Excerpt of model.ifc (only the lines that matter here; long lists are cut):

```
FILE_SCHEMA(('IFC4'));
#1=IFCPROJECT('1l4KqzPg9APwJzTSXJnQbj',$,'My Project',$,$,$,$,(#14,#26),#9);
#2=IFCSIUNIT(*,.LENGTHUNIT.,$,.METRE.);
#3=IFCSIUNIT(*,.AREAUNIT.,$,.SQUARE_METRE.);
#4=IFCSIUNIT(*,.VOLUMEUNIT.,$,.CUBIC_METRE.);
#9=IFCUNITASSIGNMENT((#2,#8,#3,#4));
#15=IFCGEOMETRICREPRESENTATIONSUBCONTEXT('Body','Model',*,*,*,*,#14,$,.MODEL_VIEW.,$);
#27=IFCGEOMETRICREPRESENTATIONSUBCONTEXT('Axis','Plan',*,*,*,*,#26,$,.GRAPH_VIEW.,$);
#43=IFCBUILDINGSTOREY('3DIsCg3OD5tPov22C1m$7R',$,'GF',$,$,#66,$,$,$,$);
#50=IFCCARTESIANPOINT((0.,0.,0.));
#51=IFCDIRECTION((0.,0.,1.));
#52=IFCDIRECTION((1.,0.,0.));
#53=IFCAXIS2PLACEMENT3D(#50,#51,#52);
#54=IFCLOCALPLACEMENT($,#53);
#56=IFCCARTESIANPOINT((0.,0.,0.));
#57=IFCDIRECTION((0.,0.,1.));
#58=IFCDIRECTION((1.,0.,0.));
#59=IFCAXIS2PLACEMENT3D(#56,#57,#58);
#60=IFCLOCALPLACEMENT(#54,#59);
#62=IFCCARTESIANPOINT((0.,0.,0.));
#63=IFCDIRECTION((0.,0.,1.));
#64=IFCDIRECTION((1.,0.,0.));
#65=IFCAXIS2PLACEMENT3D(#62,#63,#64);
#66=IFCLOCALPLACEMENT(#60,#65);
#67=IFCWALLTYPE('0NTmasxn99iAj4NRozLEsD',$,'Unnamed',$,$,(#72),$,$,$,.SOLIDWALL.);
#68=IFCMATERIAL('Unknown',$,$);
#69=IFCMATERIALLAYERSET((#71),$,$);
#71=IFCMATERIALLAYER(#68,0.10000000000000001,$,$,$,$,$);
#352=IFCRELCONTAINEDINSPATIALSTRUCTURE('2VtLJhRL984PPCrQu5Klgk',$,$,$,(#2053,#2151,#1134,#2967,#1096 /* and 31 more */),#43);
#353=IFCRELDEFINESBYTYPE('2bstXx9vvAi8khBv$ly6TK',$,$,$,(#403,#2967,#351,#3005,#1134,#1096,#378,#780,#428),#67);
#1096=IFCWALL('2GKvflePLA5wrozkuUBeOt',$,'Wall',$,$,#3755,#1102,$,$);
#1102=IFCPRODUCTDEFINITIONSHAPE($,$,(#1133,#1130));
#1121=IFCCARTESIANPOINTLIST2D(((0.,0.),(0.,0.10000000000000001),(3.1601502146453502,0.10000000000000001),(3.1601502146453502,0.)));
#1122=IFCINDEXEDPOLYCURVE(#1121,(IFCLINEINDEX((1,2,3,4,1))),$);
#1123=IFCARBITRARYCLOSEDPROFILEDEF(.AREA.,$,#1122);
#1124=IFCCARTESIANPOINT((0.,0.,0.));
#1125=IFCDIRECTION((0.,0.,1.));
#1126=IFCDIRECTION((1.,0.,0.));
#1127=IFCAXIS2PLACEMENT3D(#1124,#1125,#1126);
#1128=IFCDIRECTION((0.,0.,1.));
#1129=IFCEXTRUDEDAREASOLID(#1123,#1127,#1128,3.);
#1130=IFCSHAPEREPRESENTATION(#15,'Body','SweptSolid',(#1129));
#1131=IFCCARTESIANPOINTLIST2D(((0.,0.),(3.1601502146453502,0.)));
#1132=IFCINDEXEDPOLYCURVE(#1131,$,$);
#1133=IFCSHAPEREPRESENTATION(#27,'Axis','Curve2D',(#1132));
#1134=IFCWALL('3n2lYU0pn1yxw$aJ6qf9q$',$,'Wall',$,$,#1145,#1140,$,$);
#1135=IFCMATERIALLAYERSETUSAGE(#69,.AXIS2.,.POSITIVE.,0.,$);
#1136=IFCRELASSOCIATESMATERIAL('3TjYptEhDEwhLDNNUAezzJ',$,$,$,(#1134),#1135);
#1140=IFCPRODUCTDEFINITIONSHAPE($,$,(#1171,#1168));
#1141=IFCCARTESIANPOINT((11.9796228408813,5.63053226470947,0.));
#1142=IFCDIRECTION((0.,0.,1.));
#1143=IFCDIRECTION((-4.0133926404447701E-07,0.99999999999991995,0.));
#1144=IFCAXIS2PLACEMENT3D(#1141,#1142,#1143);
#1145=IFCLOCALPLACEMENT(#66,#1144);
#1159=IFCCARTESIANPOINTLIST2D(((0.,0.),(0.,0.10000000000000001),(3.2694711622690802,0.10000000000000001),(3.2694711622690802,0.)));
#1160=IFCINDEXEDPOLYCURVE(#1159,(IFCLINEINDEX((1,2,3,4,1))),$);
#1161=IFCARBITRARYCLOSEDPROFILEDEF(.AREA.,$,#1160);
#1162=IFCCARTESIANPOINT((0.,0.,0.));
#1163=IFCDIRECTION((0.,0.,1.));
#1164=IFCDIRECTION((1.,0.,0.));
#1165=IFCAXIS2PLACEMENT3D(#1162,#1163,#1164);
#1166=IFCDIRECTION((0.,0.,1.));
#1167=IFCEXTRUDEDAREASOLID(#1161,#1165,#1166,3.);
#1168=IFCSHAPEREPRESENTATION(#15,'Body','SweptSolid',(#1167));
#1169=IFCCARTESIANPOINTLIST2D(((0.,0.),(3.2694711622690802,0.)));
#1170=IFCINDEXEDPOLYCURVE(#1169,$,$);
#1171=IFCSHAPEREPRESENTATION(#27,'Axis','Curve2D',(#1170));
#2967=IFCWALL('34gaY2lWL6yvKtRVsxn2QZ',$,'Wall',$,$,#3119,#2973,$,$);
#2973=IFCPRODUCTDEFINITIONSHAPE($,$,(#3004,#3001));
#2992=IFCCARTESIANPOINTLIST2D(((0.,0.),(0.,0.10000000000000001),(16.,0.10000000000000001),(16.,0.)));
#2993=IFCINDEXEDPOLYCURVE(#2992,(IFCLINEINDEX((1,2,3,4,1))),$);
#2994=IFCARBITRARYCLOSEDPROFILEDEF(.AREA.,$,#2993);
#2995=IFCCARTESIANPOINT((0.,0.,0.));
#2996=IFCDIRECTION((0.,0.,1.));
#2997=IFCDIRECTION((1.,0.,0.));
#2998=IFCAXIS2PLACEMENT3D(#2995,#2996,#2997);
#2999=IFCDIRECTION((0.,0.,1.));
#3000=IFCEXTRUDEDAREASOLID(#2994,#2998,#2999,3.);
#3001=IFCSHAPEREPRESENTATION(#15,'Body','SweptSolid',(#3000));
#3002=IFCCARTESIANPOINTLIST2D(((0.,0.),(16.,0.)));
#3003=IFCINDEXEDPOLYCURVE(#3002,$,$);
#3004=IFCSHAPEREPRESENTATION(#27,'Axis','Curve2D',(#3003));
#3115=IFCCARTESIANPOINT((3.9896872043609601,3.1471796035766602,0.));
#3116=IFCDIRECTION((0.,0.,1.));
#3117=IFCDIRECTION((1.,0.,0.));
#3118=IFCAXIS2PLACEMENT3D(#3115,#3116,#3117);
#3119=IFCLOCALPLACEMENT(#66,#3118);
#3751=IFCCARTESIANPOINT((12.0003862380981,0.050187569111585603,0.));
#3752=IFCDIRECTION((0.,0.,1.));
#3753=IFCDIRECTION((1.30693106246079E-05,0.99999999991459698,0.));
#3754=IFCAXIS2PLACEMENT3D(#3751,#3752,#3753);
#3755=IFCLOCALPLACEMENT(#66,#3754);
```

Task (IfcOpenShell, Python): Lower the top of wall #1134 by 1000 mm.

```python
import ifcopenshell
import ifcopenshell.geom
import ifcopenshell.util.representation
import ifcopenshell.util.shape
import ifcopenshell.util.unit

model = ifcopenshell.open("model.ifc")
unit_scale = ifcopenshell.util.unit.calculate_unit_scale(model)
settings = ifcopenshell.geom.settings()


def volume(element):
    """Net volume in cubic metres, openings subtracted."""
    shape = ifcopenshell.geom.create_shape(settings, element)
    return ifcopenshell.util.shape.get_volume(shape.geometry)


wall = model.by_id(1134)
before = volume(wall)

body = ifcopenshell.util.representation.get_representation(wall, "Model", "Body")
solid = body.Items[0]
old_height = solid.Depth
solid.Depth -= 1 / unit_scale
after = volume(wall)

print(f"height {old_height:g} -> {solid.Depth:g}, volume {before:.3f} -> {after:.3f} m3")

model.write("model_v2.ifc")
```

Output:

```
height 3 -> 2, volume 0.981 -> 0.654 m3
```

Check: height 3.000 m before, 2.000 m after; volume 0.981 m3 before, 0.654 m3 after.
